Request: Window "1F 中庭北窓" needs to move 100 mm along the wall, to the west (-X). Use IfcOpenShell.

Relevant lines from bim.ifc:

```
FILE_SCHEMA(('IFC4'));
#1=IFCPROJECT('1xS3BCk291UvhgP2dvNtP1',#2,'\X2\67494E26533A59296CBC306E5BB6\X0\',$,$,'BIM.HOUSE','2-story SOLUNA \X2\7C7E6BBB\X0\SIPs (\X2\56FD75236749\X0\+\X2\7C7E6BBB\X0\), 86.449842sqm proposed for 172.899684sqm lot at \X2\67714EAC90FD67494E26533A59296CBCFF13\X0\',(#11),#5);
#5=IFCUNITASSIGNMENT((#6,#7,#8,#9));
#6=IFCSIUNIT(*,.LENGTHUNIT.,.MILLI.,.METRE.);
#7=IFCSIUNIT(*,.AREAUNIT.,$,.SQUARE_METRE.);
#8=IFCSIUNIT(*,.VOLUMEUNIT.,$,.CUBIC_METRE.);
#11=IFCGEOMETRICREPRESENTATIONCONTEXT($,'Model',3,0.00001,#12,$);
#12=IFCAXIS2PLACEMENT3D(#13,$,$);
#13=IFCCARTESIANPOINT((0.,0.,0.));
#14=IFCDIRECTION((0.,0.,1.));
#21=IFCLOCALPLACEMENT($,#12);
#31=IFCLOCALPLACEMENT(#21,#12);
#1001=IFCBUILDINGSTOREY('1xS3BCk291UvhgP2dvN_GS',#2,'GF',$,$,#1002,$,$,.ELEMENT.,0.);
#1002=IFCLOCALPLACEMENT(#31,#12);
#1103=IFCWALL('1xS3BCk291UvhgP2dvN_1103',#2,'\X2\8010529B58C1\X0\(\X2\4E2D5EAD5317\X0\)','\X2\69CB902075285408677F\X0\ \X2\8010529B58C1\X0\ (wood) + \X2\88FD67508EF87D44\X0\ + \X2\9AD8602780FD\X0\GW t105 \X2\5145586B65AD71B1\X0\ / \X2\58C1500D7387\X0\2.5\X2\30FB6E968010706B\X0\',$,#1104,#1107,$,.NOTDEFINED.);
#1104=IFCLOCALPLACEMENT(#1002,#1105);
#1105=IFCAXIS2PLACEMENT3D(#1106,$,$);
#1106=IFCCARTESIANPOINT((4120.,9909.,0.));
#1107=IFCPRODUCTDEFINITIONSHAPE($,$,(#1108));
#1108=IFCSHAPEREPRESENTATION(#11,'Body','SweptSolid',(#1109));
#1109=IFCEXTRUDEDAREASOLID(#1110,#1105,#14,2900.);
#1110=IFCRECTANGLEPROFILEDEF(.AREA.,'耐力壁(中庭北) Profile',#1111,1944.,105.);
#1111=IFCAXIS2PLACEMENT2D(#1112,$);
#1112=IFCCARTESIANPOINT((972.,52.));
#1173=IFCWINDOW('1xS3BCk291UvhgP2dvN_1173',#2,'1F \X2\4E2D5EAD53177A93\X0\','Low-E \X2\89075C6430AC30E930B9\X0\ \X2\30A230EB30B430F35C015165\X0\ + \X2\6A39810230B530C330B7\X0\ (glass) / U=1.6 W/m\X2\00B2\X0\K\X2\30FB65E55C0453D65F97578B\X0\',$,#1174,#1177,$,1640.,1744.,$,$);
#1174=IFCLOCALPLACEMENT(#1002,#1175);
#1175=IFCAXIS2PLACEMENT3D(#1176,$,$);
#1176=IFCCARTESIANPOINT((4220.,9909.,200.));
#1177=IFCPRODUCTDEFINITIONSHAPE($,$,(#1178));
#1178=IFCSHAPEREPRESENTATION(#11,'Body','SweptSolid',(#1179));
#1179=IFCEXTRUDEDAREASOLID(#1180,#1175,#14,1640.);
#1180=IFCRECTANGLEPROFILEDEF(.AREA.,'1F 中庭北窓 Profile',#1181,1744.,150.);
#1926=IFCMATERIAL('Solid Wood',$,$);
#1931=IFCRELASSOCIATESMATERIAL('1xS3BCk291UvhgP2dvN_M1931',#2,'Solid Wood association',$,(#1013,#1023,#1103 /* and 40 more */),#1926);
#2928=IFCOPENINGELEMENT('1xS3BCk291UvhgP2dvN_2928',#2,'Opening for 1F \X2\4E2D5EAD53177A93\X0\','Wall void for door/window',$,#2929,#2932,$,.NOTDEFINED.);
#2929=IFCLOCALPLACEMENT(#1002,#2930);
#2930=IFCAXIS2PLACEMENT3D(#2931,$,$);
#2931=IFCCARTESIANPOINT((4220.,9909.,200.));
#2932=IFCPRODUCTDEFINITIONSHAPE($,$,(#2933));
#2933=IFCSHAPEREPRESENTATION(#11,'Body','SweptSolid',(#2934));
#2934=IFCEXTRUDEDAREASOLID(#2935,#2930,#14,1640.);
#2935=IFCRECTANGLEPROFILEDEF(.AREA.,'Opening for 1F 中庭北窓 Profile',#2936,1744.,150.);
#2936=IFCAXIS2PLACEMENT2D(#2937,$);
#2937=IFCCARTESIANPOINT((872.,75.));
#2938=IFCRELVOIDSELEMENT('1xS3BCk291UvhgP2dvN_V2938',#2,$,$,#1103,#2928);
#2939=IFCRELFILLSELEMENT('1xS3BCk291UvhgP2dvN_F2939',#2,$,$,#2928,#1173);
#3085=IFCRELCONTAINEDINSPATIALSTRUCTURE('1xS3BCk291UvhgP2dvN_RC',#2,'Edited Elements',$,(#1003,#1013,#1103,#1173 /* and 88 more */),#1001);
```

```python
import ifcopenshell
import ifcopenshell.api.geometry
import ifcopenshell.util.placement
import ifcopenshell.util.unit

model = ifcopenshell.open("bim.ifc")
unit_scale = ifcopenshell.util.unit.calculate_unit_scale(model)

window = model.by_guid("1xS3BCk291UvhgP2dvN_1173")
opening = window.FillsVoids[0].RelatingOpeningElement
wall = opening.VoidsElements[0].RelatingBuildingElement

wall_matrix = ifcopenshell.util.placement.get_local_placement(wall.ObjectPlacement)
shift = wall_matrix[:3, 0] * -0.1 / unit_scale
before = ifcopenshell.util.placement.get_local_placement(window.ObjectPlacement)[:3, 3].copy()

# The window is not placed relative to its opening, so move both.
for product in (opening, window):
    matrix = ifcopenshell.util.placement.get_local_placement(product.ObjectPlacement)
    matrix[:3, 3] += shift
    ifcopenshell.api.geometry.edit_object_placement(model, product=product, matrix=matrix, is_si=False)

after = ifcopenshell.util.placement.get_local_placement(window.ObjectPlacement)[:3, 3]
print("window moved by", (after - before).round(3) + 0.0)

model.write("bim_v2.ifc")
```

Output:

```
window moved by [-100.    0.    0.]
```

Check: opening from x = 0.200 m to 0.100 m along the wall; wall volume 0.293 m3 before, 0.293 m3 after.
